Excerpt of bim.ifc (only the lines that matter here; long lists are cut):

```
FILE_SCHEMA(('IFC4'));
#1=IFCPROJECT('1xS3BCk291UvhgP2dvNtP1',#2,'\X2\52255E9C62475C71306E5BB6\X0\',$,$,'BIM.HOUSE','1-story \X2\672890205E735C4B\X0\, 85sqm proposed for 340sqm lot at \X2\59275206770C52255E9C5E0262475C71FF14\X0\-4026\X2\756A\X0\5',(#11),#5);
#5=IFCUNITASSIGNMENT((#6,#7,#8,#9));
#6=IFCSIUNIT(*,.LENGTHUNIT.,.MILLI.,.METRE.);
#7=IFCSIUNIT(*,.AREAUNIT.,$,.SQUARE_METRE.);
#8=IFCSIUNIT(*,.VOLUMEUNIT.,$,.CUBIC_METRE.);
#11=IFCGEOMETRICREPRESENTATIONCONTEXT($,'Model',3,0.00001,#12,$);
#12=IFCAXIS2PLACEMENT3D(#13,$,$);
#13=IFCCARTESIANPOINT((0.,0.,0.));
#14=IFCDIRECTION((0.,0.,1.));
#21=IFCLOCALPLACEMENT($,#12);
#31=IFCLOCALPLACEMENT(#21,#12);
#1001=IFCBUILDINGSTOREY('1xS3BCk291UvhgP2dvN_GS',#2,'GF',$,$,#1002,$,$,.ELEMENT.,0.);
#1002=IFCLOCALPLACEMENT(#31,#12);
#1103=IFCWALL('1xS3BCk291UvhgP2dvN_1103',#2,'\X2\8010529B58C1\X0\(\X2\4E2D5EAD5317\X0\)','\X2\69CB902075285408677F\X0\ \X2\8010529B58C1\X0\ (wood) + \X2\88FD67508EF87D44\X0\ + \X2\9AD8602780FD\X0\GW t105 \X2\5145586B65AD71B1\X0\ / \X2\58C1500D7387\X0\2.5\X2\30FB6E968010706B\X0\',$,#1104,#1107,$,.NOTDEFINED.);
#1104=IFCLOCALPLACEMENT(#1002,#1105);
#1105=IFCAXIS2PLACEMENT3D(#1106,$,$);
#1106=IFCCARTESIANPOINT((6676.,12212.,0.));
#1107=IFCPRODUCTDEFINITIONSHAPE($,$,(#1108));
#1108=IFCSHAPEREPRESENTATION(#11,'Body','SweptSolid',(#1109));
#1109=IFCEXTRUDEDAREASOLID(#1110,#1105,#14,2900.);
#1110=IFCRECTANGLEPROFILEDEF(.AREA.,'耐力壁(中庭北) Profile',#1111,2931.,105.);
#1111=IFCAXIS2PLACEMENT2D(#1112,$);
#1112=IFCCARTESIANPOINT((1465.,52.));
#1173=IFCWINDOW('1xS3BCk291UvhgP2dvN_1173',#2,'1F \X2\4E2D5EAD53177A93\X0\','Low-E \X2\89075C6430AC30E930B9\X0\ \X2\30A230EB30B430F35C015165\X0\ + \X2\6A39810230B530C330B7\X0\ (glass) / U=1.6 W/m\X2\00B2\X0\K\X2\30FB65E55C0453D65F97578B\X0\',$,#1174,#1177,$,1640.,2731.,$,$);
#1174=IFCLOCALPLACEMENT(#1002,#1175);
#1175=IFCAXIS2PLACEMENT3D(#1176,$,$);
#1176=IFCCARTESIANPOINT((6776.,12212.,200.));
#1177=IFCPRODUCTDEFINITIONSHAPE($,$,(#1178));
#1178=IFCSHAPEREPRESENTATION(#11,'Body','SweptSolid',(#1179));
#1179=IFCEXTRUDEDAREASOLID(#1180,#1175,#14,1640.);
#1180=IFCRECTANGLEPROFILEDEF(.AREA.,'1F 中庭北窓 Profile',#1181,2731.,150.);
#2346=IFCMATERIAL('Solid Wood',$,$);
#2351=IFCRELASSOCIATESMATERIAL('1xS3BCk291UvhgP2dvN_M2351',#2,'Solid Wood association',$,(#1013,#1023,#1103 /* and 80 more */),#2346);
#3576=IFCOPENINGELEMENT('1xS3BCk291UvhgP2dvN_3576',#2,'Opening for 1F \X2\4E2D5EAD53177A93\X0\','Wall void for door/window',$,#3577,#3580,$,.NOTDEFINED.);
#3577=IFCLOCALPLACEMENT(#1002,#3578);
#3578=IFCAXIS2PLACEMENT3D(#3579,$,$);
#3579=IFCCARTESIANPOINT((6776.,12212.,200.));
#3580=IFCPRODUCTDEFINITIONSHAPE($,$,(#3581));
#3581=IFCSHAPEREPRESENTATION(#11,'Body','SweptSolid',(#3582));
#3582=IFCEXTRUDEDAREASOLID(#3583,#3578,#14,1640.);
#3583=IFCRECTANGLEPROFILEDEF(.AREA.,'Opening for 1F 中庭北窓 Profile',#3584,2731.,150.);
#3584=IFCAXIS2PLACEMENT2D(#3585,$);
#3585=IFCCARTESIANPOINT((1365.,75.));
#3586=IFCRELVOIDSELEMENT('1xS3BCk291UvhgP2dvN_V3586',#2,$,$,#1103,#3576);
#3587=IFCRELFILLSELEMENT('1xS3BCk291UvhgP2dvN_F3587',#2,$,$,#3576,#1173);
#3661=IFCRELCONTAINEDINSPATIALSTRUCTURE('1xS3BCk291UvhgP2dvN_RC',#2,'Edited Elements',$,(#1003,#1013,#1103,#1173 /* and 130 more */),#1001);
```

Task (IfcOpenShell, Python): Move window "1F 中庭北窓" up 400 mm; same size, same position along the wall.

```python
import numpy as np
import ifcopenshell
import ifcopenshell.api.geometry
import ifcopenshell.util.placement
import ifcopenshell.util.unit

model = ifcopenshell.open("bim.ifc")
unit_scale = ifcopenshell.util.unit.calculate_unit_scale(model)

window = model.by_guid("1xS3BCk291UvhgP2dvN_1173")
opening = window.FillsVoids[0].RelatingOpeningElement
dz = 0.4 / unit_scale

shift = np.array([0.0, 0.0, dz])
# The window is not placed relative to its opening, so move both.
for product in (opening, window):
    matrix = ifcopenshell.util.placement.get_local_placement(product.ObjectPlacement)
    matrix[:3, 3] += shift
    ifcopenshell.api.geometry.edit_object_placement(model, product=product, matrix=matrix, is_si=False)

print(f"moved by {dz * unit_scale:+.3f} m")

model.write("bim-out.ifc")
```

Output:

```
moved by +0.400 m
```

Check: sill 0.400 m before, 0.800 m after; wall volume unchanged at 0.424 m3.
